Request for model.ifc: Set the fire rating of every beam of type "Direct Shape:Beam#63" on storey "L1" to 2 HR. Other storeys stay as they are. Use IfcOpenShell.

First a look at what the model holds.

```python
import ifcopenshell
import ifcopenshell.util.element

model = ifcopenshell.open("model.ifc")
print(model.schema)
storey = next(s for s in model.by_type("IfcBuildingStorey") if s.Name == "L1")
beams = [e for e in ifcopenshell.util.element.get_decomposition(storey) if e.is_a("IfcBeam")]
seen = {}
for e in beams:
    element_type = ifcopenshell.util.element.get_type(e)
    key = (element_type.Name if element_type != e and element_type else None, ifcopenshell.util.element.get_pset(e, "Pset_BeamCommon", "FireRating"))
    seen[key] = seen.get(key, 0) + 1
for (name, value), count in sorted(seen.items(), key=str):
    print(count, "x", name, "|", value)
```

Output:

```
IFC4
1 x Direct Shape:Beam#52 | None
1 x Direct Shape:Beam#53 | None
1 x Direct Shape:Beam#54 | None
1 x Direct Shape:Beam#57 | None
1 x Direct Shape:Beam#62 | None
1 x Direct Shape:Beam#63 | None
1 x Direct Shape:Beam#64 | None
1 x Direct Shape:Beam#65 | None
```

```python
import ifcopenshell
import ifcopenshell.api.pset
import ifcopenshell.util.element

model = ifcopenshell.open("model.ifc")

storey = next(s for s in model.by_type("IfcBuildingStorey") if s.Name == "L1")
beams = [e for e in ifcopenshell.util.element.get_decomposition(storey) if e.is_a("IfcBeam")]

count = 0
for e in beams:
    element_type = ifcopenshell.util.element.get_type(e)
    if element_type in (None, e) or element_type.Name != "Direct Shape:Beam#63":
        continue
    # add_pset returns the element's existing set when there is one.
    pset = ifcopenshell.api.pset.add_pset(model, product=e, name="Pset_BeamCommon")
    ifcopenshell.api.pset.edit_pset(model, pset=pset, properties={"FireRating": "2 HR"})
    count += 1

print(count, "beams updated")

model.write("model_v2.ifc")
```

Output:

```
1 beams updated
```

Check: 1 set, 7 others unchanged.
